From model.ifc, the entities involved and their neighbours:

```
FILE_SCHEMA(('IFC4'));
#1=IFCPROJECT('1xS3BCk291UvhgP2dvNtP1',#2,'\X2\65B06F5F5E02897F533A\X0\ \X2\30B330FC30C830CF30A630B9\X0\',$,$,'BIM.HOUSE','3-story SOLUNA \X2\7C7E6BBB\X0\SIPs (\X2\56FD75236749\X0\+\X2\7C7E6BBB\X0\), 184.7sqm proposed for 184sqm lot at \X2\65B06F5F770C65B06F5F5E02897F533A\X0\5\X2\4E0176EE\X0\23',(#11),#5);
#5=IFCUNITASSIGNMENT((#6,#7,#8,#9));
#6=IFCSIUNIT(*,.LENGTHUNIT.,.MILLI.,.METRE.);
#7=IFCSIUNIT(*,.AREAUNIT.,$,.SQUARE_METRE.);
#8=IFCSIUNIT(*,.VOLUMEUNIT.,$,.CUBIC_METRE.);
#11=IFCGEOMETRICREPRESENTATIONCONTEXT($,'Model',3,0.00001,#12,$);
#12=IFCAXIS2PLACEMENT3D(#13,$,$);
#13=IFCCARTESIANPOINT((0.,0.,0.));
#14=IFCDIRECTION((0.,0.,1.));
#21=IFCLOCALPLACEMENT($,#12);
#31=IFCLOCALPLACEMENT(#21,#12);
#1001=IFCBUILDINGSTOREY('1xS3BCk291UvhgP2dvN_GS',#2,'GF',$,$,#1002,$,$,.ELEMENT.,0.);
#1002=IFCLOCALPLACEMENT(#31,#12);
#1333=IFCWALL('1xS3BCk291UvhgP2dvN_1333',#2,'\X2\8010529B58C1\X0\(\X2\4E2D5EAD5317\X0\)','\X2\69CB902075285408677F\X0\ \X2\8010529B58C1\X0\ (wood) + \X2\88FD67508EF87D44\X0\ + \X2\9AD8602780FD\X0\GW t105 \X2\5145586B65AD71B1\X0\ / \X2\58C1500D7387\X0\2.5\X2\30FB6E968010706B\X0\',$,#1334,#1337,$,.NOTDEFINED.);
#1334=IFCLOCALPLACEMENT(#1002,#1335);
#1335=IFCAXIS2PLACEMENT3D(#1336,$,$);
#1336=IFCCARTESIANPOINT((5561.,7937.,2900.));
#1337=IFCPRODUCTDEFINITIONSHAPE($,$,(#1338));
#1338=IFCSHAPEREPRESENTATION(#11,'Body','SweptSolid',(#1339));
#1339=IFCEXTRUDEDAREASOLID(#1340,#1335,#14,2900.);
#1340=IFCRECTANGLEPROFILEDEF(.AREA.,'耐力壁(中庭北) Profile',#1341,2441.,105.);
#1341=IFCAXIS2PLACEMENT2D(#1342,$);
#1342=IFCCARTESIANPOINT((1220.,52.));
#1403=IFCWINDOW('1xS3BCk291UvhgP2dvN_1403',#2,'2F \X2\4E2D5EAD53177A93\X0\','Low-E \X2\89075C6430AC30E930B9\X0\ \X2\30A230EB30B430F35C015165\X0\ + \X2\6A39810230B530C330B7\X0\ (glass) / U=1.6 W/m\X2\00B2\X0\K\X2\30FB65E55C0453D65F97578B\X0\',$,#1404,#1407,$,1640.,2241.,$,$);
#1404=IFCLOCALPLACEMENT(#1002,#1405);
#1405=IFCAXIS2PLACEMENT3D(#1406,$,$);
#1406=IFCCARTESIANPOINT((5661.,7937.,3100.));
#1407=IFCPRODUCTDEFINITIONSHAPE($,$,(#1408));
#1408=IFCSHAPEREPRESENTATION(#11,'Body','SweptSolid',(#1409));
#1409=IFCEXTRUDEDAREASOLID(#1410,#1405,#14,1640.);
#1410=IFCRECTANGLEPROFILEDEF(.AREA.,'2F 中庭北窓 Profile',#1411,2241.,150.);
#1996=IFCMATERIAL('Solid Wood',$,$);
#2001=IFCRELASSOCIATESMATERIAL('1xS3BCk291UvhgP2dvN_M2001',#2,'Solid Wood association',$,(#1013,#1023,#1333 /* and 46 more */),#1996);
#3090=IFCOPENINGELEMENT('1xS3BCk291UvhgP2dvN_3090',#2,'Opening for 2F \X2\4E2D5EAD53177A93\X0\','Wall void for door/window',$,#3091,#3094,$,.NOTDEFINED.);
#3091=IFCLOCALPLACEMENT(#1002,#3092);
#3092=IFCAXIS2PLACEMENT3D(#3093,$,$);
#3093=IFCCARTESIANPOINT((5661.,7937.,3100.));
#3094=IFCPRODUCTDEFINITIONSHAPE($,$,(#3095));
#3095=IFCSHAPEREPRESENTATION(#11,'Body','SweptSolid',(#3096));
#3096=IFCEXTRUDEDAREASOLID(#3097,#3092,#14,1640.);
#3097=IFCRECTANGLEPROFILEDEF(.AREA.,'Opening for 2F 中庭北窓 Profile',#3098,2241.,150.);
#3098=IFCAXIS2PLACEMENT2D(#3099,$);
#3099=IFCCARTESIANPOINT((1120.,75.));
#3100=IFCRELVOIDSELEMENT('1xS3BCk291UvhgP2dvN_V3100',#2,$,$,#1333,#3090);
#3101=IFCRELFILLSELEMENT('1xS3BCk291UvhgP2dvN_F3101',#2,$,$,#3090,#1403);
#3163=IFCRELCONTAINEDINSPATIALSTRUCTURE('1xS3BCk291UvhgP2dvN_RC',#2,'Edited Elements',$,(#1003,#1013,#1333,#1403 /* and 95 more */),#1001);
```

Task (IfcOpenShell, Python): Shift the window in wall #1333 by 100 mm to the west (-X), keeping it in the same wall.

```python
import ifcopenshell
import ifcopenshell.api.geometry
import ifcopenshell.util.placement

model = ifcopenshell.open("model.ifc")

window = model.by_guid("1xS3BCk291UvhgP2dvN_1403")
opening = window.FillsVoids[0].RelatingOpeningElement
wall = opening.VoidsElements[0].RelatingBuildingElement

wall_matrix = ifcopenshell.util.placement.get_local_placement(wall.ObjectPlacement)
shift = wall_matrix[:3, 0] * -100.0
before = ifcopenshell.util.placement.get_local_placement(window.ObjectPlacement)[:3, 3].copy()

# The window is not placed relative to its opening, so move both.
for product in (opening, window):
    matrix = ifcopenshell.util.placement.get_local_placement(product.ObjectPlacement)
    matrix[:3, 3] += shift
    ifcopenshell.api.geometry.edit_object_placement(model, product=product, matrix=matrix, is_si=False)

after = ifcopenshell.util.placement.get_local_placement(window.ObjectPlacement)[:3, 3]
print("window moved by", (after - before).round(3) + 0.0)

model.write("model_updated.ifc")
```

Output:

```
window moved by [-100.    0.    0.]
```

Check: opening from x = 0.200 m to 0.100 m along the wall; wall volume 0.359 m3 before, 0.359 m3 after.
